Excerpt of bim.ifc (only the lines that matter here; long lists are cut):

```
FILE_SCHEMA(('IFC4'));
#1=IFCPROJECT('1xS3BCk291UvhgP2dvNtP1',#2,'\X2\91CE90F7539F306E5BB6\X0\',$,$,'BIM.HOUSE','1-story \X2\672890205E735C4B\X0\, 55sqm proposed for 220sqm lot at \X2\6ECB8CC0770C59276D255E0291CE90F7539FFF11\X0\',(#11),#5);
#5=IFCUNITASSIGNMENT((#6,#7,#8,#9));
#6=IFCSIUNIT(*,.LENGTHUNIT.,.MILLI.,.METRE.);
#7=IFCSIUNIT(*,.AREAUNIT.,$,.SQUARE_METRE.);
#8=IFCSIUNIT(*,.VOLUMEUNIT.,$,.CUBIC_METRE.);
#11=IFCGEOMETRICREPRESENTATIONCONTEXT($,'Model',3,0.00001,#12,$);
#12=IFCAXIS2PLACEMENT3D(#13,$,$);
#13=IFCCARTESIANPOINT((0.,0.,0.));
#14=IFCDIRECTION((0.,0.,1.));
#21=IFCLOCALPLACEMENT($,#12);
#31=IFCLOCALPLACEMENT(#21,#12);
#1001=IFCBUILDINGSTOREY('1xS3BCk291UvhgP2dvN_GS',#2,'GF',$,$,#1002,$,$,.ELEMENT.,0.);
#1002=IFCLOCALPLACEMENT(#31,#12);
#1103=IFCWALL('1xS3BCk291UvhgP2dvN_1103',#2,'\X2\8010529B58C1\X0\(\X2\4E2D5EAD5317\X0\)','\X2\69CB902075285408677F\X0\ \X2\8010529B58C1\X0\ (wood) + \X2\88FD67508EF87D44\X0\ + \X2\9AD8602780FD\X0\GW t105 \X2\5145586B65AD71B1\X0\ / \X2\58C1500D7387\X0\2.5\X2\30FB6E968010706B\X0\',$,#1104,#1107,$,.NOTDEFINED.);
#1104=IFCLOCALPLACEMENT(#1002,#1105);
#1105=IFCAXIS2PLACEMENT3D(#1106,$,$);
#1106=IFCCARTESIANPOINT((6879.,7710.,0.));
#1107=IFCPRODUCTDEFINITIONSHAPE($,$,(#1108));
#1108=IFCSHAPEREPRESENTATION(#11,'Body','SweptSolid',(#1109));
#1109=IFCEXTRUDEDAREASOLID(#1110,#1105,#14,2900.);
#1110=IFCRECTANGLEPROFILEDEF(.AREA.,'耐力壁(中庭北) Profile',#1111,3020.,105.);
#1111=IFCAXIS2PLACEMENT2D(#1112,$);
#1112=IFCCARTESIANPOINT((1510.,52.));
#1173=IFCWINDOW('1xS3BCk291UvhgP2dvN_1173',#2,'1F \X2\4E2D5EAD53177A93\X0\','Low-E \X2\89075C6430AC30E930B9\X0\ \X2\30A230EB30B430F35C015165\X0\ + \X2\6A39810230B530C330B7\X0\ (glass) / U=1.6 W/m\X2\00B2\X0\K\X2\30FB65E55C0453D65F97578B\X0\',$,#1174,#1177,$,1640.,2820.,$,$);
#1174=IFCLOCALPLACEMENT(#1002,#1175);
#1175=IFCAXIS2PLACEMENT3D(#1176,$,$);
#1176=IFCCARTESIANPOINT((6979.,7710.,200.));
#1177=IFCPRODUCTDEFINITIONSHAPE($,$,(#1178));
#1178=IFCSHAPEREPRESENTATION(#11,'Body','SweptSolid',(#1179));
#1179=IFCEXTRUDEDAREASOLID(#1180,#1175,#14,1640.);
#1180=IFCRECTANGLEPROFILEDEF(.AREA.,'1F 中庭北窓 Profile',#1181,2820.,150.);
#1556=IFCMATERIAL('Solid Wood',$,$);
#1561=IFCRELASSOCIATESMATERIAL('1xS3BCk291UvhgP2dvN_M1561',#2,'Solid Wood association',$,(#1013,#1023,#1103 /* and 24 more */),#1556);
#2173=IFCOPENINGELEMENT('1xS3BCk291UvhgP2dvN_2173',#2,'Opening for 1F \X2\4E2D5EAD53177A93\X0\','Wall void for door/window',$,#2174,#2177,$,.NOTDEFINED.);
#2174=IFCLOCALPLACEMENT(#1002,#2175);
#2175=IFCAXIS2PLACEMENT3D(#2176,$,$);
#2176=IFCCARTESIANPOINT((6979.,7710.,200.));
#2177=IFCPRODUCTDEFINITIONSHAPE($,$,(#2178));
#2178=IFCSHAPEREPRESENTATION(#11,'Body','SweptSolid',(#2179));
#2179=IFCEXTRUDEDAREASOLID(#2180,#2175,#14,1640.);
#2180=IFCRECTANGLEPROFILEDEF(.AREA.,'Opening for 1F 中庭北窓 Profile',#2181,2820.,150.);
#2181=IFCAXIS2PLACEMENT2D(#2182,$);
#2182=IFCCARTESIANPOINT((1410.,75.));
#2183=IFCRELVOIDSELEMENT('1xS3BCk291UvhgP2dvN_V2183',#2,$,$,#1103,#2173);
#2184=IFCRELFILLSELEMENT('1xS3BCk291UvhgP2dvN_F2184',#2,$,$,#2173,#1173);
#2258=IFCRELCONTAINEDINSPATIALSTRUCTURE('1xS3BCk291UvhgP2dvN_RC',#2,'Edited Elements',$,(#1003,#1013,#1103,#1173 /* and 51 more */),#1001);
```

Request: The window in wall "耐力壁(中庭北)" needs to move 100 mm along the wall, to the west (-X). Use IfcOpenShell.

```python
import ifcopenshell
import ifcopenshell.api.geometry
import ifcopenshell.util.placement

model = ifcopenshell.open("bim.ifc")

window = model.by_guid("1xS3BCk291UvhgP2dvN_1173")
opening = window.FillsVoids[0].RelatingOpeningElement
wall = opening.VoidsElements[0].RelatingBuildingElement

wall_matrix = ifcopenshell.util.placement.get_local_placement(wall.ObjectPlacement)
shift = wall_matrix[:3, 0] * -100.0
before = ifcopenshell.util.placement.get_local_placement(window.ObjectPlacement)[:3, 3].copy()

# The window is not placed relative to its opening, so move both.
for product in (opening, window):
    matrix = ifcopenshell.util.placement.get_local_placement(product.ObjectPlacement)
    matrix[:3, 3] += shift
    ifcopenshell.api.geometry.edit_object_placement(model, product=product, matrix=matrix, is_si=False)

after = ifcopenshell.util.placement.get_local_placement(window.ObjectPlacement)[:3, 3]
print("window moved by", (after - before).round(3) + 0.0)

model.write("bim_rev.ifc")
```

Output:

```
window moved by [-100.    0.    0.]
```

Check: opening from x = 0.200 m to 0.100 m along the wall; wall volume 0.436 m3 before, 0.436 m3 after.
